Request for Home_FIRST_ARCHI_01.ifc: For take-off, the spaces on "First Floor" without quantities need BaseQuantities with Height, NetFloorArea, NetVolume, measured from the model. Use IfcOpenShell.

First a look at what the model holds.

```python
import ifcopenshell
import ifcopenshell.util.element
import ifcopenshell.util.unit

model = ifcopenshell.open("Home_FIRST_ARCHI_01.ifc")
print(model.schema)
for unit_type in ("LENGTHUNIT", "AREAUNIT", "VOLUMEUNIT"):
    print(unit_type, ifcopenshell.util.unit.calculate_unit_scale(model, unit_type))
storey = next(s for s in model.by_type("IfcBuildingStorey") if s.Name == "First Floor")
spaces = [e for e in ifcopenshell.util.element.get_decomposition(storey) if e.is_a("IfcSpace")]
for e in sorted(spaces, key=lambda e: e.id()):
    print(e.id(), e.is_a(), e.Name, list(ifcopenshell.util.element.get_psets(e, qtos_only=True)), sep=" | ")
```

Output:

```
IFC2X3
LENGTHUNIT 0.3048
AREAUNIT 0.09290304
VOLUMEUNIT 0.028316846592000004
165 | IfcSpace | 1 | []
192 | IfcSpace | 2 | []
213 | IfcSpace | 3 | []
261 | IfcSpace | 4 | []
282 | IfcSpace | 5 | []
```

```python
import ifcopenshell
import ifcopenshell.api.pset
import ifcopenshell.geom
import ifcopenshell.util.element
import ifcopenshell.util.shape
import ifcopenshell.util.unit

model = ifcopenshell.open("Home_FIRST_ARCHI_01.ifc")
unit_scale = ifcopenshell.util.unit.calculate_unit_scale(model)
area_scale = ifcopenshell.util.unit.calculate_unit_scale(model, "AREAUNIT")
volume_scale = ifcopenshell.util.unit.calculate_unit_scale(model, "VOLUMEUNIT")
settings = ifcopenshell.geom.settings()

storey = next(s for s in model.by_type("IfcBuildingStorey") if s.Name == "First Floor")
spaces = [e for e in ifcopenshell.util.element.get_decomposition(storey) if e.is_a("IfcSpace")]

for e in sorted(spaces, key=lambda e: e.id()):
    if ifcopenshell.util.element.get_psets(e, qtos_only=True, should_inherit=False):
        continue
    # Geometry comes back in metres, in the element's own axes.
    shape = ifcopenshell.geom.create_shape(settings, e)
    values = {
        "Height": ifcopenshell.util.shape.get_z(shape.geometry) / unit_scale,
        "NetFloorArea": ifcopenshell.util.shape.get_footprint_area(shape.geometry) / area_scale,
        "NetVolume": ifcopenshell.util.shape.get_volume(shape.geometry) / volume_scale,
    }
    qto = ifcopenshell.api.pset.add_qto(model, product=e, name="BaseQuantities")
    ifcopenshell.api.pset.edit_qto(model, qto=qto, properties=values)
    print(e.id(), {k: round(v, 3) for k, v in values.items()})

model.write("Home_FIRST_ARCHI_01_rev.ifc")
```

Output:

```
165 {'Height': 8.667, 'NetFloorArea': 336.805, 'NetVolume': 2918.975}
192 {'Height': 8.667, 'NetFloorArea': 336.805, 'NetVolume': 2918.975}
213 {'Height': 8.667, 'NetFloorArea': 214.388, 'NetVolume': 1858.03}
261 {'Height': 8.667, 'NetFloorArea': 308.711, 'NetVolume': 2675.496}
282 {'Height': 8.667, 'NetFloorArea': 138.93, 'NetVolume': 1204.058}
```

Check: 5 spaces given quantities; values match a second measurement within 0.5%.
